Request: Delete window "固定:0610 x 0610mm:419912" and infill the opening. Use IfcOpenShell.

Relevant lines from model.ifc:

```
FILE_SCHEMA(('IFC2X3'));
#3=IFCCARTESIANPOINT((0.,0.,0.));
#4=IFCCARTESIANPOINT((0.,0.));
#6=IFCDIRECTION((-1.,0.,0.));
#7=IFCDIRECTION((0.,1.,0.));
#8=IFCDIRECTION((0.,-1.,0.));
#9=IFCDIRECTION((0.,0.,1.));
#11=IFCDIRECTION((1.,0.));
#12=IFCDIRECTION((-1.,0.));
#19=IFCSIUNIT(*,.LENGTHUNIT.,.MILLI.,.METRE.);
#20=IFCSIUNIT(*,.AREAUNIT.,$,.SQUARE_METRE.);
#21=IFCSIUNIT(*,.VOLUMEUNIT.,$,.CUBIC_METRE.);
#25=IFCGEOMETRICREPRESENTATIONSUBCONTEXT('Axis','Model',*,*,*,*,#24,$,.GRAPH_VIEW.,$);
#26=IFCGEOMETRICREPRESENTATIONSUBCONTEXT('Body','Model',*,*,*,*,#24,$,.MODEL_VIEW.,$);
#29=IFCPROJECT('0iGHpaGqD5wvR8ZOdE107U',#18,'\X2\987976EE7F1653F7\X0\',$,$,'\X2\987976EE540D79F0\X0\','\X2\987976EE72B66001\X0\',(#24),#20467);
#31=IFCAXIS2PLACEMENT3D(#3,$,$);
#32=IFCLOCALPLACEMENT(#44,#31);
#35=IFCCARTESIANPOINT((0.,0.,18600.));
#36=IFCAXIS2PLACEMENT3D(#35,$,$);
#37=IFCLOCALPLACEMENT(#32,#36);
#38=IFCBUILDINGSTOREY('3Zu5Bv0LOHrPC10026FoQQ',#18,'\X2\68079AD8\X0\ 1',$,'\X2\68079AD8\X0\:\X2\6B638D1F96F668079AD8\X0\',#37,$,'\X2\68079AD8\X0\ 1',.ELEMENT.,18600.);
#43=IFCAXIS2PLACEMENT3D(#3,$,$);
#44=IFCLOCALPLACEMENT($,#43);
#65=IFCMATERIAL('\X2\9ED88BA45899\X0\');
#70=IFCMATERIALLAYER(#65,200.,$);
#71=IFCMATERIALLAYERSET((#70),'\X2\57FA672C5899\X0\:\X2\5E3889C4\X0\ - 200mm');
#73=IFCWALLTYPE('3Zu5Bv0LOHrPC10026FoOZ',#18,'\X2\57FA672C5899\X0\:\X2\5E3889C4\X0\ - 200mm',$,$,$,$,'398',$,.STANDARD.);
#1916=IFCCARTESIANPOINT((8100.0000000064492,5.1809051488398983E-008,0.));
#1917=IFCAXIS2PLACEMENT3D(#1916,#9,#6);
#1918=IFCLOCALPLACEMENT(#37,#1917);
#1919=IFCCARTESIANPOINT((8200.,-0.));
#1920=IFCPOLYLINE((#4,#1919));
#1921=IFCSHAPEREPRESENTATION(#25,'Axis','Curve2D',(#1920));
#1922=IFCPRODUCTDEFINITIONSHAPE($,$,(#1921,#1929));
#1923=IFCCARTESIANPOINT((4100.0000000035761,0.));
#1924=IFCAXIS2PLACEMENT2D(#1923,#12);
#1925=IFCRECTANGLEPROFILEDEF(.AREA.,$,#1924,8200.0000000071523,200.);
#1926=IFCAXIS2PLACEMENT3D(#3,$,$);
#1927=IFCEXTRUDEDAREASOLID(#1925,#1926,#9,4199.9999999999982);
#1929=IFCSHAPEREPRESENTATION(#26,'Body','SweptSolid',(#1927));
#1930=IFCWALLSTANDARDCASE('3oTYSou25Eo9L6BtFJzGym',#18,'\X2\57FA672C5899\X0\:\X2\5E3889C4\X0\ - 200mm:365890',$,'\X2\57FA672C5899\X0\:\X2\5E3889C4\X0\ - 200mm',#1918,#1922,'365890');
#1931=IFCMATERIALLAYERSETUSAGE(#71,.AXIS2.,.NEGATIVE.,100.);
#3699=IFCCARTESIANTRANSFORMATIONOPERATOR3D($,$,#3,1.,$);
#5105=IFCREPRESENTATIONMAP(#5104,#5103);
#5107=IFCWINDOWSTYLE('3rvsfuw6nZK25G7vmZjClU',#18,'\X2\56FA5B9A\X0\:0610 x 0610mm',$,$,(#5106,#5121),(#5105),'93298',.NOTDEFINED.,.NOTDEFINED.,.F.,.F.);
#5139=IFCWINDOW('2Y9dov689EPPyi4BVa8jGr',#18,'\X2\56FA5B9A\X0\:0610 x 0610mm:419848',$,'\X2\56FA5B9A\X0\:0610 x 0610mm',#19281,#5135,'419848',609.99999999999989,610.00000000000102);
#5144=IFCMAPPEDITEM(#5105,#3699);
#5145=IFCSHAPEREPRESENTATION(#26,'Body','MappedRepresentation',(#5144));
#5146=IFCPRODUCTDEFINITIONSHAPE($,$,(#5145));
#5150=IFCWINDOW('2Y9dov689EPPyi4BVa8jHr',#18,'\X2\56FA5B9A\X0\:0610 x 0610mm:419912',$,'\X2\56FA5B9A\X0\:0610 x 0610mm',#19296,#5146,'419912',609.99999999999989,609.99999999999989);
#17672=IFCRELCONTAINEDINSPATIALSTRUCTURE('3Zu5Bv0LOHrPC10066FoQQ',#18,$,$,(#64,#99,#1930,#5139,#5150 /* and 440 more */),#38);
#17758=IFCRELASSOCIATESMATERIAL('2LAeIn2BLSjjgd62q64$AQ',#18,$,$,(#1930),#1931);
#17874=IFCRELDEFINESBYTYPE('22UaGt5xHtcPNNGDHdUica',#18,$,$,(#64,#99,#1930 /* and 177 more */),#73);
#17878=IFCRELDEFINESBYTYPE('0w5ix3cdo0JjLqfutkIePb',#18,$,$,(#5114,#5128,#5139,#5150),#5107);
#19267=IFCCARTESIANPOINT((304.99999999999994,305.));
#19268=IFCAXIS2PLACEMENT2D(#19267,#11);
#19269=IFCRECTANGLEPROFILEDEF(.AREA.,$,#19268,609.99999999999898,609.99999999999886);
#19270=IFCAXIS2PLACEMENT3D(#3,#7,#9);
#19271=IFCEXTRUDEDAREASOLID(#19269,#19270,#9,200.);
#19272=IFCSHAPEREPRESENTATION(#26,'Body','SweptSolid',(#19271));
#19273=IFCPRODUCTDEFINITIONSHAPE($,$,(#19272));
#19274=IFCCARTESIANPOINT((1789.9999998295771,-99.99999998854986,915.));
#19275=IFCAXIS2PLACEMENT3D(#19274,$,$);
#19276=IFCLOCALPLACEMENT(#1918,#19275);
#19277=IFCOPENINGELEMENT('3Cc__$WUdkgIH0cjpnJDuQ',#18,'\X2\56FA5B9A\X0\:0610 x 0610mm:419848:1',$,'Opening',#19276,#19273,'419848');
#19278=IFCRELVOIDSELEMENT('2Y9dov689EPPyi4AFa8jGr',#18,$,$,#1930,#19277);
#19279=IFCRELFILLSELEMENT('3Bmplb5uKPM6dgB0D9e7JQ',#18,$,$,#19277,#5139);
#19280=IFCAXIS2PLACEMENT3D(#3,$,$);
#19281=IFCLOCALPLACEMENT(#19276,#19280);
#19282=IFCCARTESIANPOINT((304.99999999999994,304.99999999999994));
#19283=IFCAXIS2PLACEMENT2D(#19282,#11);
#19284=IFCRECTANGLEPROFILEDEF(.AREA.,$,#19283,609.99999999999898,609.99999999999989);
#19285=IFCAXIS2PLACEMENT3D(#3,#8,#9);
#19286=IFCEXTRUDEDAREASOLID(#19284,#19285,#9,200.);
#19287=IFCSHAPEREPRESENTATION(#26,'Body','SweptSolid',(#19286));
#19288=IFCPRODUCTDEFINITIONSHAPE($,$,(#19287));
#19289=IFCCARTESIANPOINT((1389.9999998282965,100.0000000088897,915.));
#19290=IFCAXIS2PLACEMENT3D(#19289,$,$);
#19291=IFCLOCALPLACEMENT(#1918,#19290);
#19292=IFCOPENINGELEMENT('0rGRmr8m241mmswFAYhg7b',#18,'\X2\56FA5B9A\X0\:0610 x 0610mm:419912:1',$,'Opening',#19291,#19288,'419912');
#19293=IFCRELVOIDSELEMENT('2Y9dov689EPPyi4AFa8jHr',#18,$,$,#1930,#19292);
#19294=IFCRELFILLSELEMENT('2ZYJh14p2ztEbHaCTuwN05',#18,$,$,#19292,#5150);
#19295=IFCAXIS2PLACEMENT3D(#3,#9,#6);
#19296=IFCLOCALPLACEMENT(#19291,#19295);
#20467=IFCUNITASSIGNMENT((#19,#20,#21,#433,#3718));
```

```python
import ifcopenshell
import ifcopenshell.api.feature
import ifcopenshell.api.root
import ifcopenshell.geom
import ifcopenshell.util.shape

model = ifcopenshell.open("model.ifc")
settings = ifcopenshell.geom.settings()


def volume(element):
    """Net volume in cubic metres, openings subtracted."""
    shape = ifcopenshell.geom.create_shape(settings, element)
    return ifcopenshell.util.shape.get_volume(shape.geometry)


window = model.by_guid("2Y9dov689EPPyi4BVa8jHr")
opening = window.FillsVoids[0].RelatingOpeningElement
wall = opening.VoidsElements[0].RelatingBuildingElement
before = volume(wall)

ifcopenshell.api.root.remove_product(model, product=window)
ifcopenshell.api.feature.remove_feature(model, feature=opening)

after = volume(wall)

print(f"wall volume {before:.3f} -> {after:.3f} m3")

model.write("model-out.ifc")
```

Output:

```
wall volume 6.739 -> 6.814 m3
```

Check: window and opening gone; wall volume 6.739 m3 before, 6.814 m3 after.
